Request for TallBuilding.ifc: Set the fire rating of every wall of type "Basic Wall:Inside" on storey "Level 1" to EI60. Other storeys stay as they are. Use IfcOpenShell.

First a look at what the model holds.

```python
import ifcopenshell
import ifcopenshell.util.element

model = ifcopenshell.open("TallBuilding.ifc")
print(model.schema)
storey = next(s for s in model.by_type("IfcBuildingStorey") if s.Name == "Level 1")
walls = [e for e in ifcopenshell.util.element.get_decomposition(storey) if e.is_a("IfcWall")]
seen = {}
for e in walls:
    element_type = ifcopenshell.util.element.get_type(e)
    key = (element_type.Name if element_type != e and element_type else None, ifcopenshell.util.element.get_pset(e, "Pset_WallCommon", "FireRating"))
    seen[key] = seen.get(key, 0) + 1
for (name, value), count in sorted(seen.items(), key=str):
    print(count, "x", name, "|", value)
```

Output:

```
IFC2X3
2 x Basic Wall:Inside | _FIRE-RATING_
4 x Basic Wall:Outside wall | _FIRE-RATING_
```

```python
import ifcopenshell
import ifcopenshell.api.pset
import ifcopenshell.util.element

model = ifcopenshell.open("TallBuilding.ifc")

storey = next(s for s in model.by_type("IfcBuildingStorey") if s.Name == "Level 1")
walls = [e for e in ifcopenshell.util.element.get_decomposition(storey) if e.is_a("IfcWall")]

count = 0
for e in walls:
    element_type = ifcopenshell.util.element.get_type(e)
    if element_type in (None, e) or element_type.Name != "Basic Wall:Inside":
        continue
    # add_pset returns the element's existing set when there is one.
    pset = ifcopenshell.api.pset.add_pset(model, product=e, name="Pset_WallCommon")
    ifcopenshell.api.pset.edit_pset(model, pset=pset, properties={"FireRating": "EI60"})
    count += 1

print(count, "walls updated")

model.write("TallBuilding_edited.ifc")
```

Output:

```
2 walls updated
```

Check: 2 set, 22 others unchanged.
